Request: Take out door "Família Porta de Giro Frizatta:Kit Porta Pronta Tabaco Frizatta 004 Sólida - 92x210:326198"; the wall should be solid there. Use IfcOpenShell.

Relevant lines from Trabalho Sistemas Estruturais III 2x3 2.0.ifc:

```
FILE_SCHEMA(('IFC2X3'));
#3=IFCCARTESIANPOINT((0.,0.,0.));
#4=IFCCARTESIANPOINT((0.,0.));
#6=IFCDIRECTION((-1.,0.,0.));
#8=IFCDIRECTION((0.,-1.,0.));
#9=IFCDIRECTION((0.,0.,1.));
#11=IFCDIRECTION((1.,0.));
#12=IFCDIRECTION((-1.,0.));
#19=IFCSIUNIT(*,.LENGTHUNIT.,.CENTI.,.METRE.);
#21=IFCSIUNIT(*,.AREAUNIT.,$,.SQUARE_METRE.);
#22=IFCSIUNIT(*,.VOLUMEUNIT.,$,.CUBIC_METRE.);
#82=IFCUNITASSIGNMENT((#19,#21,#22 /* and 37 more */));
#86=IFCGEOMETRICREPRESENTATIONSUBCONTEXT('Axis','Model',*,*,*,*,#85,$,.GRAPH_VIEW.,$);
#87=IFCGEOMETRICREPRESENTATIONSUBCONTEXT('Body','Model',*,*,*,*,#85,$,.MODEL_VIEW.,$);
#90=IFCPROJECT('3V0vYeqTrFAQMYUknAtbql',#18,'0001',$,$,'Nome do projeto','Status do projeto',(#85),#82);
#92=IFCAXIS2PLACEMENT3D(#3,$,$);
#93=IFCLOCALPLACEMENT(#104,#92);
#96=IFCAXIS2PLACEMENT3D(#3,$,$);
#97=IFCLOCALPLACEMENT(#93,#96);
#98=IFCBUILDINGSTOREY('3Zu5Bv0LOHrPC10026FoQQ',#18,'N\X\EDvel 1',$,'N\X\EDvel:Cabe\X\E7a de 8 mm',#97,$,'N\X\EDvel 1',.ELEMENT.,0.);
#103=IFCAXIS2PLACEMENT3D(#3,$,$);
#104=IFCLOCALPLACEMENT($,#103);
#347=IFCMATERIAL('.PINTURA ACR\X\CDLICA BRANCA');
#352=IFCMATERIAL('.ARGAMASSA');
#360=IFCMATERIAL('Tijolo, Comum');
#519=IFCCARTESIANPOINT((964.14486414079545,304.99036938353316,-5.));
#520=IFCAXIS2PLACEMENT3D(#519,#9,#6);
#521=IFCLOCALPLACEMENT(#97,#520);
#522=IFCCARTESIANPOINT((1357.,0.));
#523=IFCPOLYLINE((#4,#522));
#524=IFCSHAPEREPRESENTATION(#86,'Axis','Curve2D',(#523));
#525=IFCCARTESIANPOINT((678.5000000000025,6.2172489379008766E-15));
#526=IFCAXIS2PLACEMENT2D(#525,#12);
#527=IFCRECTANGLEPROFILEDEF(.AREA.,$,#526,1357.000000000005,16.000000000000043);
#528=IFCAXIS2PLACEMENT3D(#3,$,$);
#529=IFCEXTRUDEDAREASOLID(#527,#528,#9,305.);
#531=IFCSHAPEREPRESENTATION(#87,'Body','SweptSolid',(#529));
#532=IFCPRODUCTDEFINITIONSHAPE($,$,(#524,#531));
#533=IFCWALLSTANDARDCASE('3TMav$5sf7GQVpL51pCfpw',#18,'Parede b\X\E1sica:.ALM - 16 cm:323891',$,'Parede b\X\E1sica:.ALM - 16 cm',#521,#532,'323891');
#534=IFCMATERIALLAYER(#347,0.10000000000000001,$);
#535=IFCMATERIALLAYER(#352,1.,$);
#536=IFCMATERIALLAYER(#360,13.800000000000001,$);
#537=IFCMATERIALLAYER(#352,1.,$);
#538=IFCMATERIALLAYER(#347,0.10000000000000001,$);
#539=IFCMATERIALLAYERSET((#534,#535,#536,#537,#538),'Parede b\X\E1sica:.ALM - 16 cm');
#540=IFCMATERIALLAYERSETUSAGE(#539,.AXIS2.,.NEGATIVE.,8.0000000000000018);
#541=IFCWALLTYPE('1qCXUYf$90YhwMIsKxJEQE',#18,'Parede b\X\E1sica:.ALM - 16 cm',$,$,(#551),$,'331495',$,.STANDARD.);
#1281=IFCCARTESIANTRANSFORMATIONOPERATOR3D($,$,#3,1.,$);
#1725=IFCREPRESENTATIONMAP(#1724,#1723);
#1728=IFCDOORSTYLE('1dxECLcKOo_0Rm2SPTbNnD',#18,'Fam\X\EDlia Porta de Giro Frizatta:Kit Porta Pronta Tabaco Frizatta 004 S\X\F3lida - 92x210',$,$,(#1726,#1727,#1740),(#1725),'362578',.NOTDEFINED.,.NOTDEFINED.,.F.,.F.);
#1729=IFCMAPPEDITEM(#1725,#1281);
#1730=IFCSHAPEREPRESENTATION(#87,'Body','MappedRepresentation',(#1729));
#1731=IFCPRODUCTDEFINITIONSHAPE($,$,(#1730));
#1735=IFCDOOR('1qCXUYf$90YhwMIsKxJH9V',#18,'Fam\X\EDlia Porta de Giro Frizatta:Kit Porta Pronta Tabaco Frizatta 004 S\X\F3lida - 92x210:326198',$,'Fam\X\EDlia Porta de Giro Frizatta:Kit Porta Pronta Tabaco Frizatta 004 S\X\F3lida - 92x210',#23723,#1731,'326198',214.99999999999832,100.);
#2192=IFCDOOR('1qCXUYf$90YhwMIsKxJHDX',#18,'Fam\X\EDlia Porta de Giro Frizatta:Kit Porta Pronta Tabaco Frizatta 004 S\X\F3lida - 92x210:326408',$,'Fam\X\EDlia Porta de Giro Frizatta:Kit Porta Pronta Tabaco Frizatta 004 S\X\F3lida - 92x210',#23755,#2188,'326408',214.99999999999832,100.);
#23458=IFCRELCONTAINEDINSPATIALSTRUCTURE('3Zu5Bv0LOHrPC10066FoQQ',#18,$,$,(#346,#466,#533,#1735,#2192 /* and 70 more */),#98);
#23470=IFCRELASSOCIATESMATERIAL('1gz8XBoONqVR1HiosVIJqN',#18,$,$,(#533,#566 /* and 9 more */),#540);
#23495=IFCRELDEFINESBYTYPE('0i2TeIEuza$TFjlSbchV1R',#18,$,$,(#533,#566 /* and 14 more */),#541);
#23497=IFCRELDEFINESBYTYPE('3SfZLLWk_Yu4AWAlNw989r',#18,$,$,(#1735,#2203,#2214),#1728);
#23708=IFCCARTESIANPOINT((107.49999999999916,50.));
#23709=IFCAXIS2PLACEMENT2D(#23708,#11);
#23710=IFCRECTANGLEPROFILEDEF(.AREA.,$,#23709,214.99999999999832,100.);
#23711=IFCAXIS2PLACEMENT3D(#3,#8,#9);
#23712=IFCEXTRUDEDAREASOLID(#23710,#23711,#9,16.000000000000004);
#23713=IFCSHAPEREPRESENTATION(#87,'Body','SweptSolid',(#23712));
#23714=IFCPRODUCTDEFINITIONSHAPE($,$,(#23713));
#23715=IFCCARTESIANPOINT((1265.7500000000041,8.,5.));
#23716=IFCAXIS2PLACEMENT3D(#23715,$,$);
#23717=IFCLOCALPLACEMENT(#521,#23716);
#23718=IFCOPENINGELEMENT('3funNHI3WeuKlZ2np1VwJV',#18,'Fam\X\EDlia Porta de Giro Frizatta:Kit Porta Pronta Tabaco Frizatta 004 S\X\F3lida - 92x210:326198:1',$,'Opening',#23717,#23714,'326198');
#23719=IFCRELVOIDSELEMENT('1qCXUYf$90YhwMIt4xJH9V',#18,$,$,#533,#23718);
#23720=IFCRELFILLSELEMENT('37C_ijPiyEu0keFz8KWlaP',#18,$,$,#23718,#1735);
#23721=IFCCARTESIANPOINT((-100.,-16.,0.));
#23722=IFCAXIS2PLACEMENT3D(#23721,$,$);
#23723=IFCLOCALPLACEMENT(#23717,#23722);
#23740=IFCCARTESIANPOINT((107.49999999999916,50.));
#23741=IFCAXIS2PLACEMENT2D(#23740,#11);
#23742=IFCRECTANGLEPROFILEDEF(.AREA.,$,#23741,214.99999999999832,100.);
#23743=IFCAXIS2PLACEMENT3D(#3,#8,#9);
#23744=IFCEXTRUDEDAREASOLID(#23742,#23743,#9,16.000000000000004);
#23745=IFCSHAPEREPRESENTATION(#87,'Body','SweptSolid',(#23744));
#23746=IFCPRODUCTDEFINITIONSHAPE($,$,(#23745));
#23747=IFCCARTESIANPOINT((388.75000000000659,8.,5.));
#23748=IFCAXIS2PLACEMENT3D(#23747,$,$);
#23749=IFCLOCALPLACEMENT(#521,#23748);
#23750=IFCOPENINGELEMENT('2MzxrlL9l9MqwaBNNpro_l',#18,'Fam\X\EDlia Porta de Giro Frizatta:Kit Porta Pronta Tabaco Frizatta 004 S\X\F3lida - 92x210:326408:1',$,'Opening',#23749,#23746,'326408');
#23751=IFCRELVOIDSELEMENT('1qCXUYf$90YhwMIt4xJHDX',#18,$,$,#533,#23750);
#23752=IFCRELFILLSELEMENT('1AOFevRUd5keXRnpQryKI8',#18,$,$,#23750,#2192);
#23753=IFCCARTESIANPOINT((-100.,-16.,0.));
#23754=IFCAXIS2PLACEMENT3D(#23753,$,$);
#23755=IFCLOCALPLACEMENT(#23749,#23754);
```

```python
import ifcopenshell
import ifcopenshell.api.feature
import ifcopenshell.api.root
import ifcopenshell.geom
import ifcopenshell.util.shape

model = ifcopenshell.open("Trabalho Sistemas Estruturais III 2x3 2.0.ifc")
settings = ifcopenshell.geom.settings()


def volume(element):
    """Net volume in cubic metres, openings subtracted."""
    shape = ifcopenshell.geom.create_shape(settings, element)
    return ifcopenshell.util.shape.get_volume(shape.geometry)


door = model.by_guid("1qCXUYf$90YhwMIsKxJH9V")
opening = door.FillsVoids[0].RelatingOpeningElement
wall = opening.VoidsElements[0].RelatingBuildingElement
before = volume(wall)

ifcopenshell.api.root.remove_product(model, product=door)
ifcopenshell.api.feature.remove_feature(model, feature=opening)

after = volume(wall)

print(f"wall volume {before:.3f} -> {after:.3f} m3")

model.write("Trabalho Sistemas Estruturais III 2x3 2.0_v2.ifc")
```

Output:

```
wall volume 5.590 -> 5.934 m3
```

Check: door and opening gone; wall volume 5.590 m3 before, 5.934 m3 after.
